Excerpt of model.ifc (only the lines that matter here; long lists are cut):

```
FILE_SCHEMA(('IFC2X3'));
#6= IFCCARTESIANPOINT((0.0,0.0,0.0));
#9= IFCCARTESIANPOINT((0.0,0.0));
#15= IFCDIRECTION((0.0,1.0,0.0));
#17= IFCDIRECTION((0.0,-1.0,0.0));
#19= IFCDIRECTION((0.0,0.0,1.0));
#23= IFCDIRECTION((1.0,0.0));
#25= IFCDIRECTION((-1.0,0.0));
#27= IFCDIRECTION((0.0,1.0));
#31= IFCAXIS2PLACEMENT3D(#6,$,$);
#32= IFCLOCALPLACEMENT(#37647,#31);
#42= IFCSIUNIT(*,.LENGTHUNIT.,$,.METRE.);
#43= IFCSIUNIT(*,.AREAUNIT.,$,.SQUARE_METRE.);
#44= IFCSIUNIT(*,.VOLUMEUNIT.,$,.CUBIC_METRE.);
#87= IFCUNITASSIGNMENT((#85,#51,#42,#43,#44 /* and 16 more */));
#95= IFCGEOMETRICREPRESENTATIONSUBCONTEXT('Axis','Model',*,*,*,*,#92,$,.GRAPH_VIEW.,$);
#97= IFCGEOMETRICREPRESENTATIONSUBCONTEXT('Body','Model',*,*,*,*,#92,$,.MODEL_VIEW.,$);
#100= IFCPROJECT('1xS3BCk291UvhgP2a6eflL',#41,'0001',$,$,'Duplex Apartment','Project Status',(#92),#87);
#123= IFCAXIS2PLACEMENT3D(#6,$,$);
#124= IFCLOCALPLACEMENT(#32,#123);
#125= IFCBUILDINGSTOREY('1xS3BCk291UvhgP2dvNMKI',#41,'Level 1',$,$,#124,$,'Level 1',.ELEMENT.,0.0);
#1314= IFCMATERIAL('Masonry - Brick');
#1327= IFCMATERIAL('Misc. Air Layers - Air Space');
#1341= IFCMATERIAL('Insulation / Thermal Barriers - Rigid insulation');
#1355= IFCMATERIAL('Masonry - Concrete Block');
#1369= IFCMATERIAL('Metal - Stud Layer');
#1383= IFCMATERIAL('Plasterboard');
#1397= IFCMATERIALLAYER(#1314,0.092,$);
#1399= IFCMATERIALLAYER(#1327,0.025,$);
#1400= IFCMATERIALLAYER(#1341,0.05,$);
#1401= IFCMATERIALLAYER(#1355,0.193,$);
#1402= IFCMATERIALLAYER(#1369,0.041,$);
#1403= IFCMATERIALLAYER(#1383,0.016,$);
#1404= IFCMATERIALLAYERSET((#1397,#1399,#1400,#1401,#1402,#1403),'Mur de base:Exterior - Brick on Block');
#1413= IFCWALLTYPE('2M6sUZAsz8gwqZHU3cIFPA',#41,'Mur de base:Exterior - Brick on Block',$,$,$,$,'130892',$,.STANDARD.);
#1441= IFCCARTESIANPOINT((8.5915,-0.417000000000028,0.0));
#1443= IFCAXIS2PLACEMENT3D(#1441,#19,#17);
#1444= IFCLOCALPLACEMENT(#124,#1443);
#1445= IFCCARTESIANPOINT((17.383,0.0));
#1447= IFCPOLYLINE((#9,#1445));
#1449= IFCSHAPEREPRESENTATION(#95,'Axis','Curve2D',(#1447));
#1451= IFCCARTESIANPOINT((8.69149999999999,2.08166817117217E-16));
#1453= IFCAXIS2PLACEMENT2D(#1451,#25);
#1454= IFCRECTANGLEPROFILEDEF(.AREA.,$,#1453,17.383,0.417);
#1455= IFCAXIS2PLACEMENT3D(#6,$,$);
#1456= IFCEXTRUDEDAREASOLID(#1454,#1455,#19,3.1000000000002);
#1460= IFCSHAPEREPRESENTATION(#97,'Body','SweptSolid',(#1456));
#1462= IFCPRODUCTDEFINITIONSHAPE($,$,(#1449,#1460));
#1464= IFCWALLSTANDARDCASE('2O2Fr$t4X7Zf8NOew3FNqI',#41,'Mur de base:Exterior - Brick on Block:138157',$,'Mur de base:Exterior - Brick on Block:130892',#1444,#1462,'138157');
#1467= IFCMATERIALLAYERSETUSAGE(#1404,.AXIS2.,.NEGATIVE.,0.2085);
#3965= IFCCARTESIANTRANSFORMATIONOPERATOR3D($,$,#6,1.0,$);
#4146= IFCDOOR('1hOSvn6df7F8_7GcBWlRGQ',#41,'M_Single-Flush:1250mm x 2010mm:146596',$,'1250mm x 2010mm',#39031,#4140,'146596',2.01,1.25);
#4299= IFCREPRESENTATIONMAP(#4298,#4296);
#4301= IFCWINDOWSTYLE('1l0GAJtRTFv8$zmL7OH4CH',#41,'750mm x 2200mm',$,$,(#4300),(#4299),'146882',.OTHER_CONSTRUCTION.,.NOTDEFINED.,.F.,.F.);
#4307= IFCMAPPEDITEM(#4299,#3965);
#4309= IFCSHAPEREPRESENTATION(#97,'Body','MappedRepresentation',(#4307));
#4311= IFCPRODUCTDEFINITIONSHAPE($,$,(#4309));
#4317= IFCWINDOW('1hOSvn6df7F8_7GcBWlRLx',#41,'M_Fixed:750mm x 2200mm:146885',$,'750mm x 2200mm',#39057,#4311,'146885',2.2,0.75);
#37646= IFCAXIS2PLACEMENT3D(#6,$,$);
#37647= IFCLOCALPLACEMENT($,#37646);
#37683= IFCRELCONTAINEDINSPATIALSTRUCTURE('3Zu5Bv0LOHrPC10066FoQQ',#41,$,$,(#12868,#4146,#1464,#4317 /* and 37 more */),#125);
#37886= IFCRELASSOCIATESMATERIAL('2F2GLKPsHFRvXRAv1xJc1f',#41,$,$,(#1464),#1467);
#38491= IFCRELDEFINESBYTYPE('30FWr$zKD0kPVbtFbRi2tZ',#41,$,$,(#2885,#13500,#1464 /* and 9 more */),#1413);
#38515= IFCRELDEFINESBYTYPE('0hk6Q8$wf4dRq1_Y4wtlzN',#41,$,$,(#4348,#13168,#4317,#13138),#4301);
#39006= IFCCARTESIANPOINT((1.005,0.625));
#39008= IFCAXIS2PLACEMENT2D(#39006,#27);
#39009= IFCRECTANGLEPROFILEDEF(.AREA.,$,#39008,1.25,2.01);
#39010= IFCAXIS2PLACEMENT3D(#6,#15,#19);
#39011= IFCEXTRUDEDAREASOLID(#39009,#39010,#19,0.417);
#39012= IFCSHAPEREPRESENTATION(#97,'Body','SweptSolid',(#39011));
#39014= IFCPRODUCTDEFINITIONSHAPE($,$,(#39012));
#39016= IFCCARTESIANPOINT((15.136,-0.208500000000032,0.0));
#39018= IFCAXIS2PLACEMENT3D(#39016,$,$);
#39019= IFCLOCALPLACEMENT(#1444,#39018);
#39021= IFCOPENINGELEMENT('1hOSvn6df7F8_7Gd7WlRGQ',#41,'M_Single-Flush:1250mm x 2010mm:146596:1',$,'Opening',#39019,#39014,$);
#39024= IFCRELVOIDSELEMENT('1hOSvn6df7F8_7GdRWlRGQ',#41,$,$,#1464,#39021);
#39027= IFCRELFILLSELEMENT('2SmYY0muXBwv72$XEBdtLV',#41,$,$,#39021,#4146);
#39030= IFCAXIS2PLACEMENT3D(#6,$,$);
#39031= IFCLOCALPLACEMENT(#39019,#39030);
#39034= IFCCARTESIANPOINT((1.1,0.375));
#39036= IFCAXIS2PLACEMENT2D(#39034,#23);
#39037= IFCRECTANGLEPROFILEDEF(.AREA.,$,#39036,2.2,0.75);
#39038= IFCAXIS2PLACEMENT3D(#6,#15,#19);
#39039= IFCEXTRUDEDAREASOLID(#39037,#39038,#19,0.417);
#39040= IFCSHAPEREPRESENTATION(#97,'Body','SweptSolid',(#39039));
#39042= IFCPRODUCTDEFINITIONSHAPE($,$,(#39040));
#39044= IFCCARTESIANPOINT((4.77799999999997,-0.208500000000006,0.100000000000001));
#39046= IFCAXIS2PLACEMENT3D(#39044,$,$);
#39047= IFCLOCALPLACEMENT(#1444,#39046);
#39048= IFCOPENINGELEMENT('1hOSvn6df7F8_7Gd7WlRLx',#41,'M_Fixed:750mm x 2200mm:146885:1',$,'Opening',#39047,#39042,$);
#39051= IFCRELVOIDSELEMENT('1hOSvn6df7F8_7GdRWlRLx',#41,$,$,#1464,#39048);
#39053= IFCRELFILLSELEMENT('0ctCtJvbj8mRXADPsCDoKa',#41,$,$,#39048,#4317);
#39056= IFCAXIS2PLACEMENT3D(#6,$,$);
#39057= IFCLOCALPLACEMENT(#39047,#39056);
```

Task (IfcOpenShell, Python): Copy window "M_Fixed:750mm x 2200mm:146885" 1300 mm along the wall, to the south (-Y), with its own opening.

```python
import ifcopenshell
import ifcopenshell.api.feature
import ifcopenshell.api.geometry
import ifcopenshell.api.root
import ifcopenshell.geom
import ifcopenshell.util.element
import ifcopenshell.util.placement
import ifcopenshell.util.shape

model = ifcopenshell.open("model.ifc")
settings = ifcopenshell.geom.settings()


def volume(element):
    """Net volume in cubic metres, openings subtracted."""
    shape = ifcopenshell.geom.create_shape(settings, element)
    return ifcopenshell.util.shape.get_volume(shape.geometry)


def reuse_history(source, copy):
    """copy_class also copies each property set's owner history, people and application; keep the originals."""
    for rel in copy.IsDefinedBy:
        if rel.is_a("IfcRelDefinesByProperties") and (history := rel.RelatingPropertyDefinition.OwnerHistory):
            rel.RelatingPropertyDefinition.OwnerHistory = source.OwnerHistory
            ifcopenshell.util.element.remove_deep2(model, history)


window = model.by_guid("1hOSvn6df7F8_7GcBWlRLx")
opening = window.FillsVoids[0].RelatingOpeningElement
wall = opening.VoidsElements[0].RelatingBuildingElement
before = volume(wall)
shift = ifcopenshell.util.placement.get_local_placement(wall.ObjectPlacement)[:3, 0] * 1.3

# copy_class copies the void relationship, type, container and properties, but no geometry.
new_opening = ifcopenshell.api.root.copy_class(model, product=opening)
new_opening.Representation = ifcopenshell.util.element.copy_deep(
    model, opening.Representation, exclude=["IfcGeometricRepresentationContext", "IfcRepresentationMap"]
)
new_opening.Name = "M_Fixed:750mm x 2200mm"
new_window = ifcopenshell.api.root.copy_class(model, product=window)
new_window.Representation = ifcopenshell.util.element.copy_deep(
    model, window.Representation, exclude=["IfcGeometricRepresentationContext", "IfcRepresentationMap"]
)
new_window.Name = "M_Fixed:750mm x 2200mm"
new_window.Tag = None
reuse_history(window, new_window)
fills = ifcopenshell.api.feature.add_filling(model, opening=new_opening, element=new_window)
fills.OwnerHistory = new_window.OwnerHistory  # required in IFC2X3

for old, new in ((opening, new_opening), (window, new_window)):
    matrix = ifcopenshell.util.placement.get_local_placement(old.ObjectPlacement)
    matrix[:3, 3] += shift
    ifcopenshell.api.geometry.edit_object_placement(model, product=new, matrix=matrix, is_si=False)

after = volume(wall)

print(f"wall volume {before:.3f} -> {after:.3f} m3")

model.write("model_rev.ifc")
```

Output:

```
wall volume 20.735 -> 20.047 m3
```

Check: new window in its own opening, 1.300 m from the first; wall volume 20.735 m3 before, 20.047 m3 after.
